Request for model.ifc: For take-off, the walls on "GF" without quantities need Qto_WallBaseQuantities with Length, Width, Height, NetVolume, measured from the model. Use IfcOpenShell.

First a look at what the model holds.

```python
import ifcopenshell
import ifcopenshell.util.element
import ifcopenshell.util.unit

model = ifcopenshell.open("model.ifc")
print(model.schema)
for unit_type in ("LENGTHUNIT", "AREAUNIT", "VOLUMEUNIT"):
    print(unit_type, ifcopenshell.util.unit.calculate_unit_scale(model, unit_type))
storey = next(s for s in model.by_type("IfcBuildingStorey") if s.Name == "GF")
walls = [e for e in ifcopenshell.util.element.get_decomposition(storey) if e.is_a("IfcWall")]
for e in sorted(walls, key=lambda e: e.id()):
    print(e.id(), e.is_a(), e.Name, list(ifcopenshell.util.element.get_psets(e, qtos_only=True)), sep=" | ")
```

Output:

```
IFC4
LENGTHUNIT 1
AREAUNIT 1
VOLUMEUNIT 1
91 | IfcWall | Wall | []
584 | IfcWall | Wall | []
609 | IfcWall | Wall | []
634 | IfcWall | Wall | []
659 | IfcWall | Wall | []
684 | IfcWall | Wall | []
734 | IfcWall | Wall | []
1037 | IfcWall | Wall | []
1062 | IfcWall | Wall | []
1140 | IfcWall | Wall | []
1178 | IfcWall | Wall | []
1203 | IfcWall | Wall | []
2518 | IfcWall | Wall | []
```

```python
import ifcopenshell
import ifcopenshell.api.pset
import ifcopenshell.geom
import ifcopenshell.util.element
import ifcopenshell.util.shape
import ifcopenshell.util.unit

model = ifcopenshell.open("model.ifc")
unit_scale = ifcopenshell.util.unit.calculate_unit_scale(model)
volume_scale = ifcopenshell.util.unit.calculate_unit_scale(model, "VOLUMEUNIT")
settings = ifcopenshell.geom.settings()

storey = next(s for s in model.by_type("IfcBuildingStorey") if s.Name == "GF")
walls = [e for e in ifcopenshell.util.element.get_decomposition(storey) if e.is_a("IfcWall")]

for e in sorted(walls, key=lambda e: e.id()):
    if ifcopenshell.util.element.get_psets(e, qtos_only=True, should_inherit=False):
        continue
    # Geometry comes back in metres, in the element's own axes.
    shape = ifcopenshell.geom.create_shape(settings, e)
    values = {
        "Length": ifcopenshell.util.shape.get_x(shape.geometry) / unit_scale,
        "Width": ifcopenshell.util.shape.get_y(shape.geometry) / unit_scale,
        "Height": ifcopenshell.util.shape.get_z(shape.geometry) / unit_scale,
        "NetVolume": ifcopenshell.util.shape.get_volume(shape.geometry) / volume_scale,
    }
    qto = ifcopenshell.api.pset.add_qto(model, product=e, name="Qto_WallBaseQuantities")
    ifcopenshell.api.pset.edit_qto(model, qto=qto, properties=values)
    print(e.id(), {k: round(v, 3) for k, v in values.items()})

model.write("model_v2.ifc")
```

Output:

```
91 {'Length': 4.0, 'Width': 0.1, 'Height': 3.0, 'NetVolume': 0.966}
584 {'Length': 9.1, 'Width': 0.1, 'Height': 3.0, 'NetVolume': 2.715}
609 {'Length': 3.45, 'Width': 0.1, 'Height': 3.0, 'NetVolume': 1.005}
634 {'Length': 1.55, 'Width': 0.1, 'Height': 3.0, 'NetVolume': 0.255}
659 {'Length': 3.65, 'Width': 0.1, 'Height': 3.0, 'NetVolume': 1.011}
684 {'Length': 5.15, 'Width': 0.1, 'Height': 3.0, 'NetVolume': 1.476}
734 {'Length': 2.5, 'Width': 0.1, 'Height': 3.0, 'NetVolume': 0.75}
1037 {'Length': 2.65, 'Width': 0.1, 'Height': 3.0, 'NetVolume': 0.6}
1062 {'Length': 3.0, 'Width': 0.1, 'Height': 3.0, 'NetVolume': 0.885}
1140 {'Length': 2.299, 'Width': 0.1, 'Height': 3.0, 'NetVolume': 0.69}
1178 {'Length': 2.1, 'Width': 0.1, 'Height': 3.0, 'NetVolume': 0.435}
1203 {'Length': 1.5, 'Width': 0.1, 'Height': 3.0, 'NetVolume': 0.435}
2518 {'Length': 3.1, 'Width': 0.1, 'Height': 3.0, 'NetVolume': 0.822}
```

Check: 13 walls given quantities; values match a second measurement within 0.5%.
